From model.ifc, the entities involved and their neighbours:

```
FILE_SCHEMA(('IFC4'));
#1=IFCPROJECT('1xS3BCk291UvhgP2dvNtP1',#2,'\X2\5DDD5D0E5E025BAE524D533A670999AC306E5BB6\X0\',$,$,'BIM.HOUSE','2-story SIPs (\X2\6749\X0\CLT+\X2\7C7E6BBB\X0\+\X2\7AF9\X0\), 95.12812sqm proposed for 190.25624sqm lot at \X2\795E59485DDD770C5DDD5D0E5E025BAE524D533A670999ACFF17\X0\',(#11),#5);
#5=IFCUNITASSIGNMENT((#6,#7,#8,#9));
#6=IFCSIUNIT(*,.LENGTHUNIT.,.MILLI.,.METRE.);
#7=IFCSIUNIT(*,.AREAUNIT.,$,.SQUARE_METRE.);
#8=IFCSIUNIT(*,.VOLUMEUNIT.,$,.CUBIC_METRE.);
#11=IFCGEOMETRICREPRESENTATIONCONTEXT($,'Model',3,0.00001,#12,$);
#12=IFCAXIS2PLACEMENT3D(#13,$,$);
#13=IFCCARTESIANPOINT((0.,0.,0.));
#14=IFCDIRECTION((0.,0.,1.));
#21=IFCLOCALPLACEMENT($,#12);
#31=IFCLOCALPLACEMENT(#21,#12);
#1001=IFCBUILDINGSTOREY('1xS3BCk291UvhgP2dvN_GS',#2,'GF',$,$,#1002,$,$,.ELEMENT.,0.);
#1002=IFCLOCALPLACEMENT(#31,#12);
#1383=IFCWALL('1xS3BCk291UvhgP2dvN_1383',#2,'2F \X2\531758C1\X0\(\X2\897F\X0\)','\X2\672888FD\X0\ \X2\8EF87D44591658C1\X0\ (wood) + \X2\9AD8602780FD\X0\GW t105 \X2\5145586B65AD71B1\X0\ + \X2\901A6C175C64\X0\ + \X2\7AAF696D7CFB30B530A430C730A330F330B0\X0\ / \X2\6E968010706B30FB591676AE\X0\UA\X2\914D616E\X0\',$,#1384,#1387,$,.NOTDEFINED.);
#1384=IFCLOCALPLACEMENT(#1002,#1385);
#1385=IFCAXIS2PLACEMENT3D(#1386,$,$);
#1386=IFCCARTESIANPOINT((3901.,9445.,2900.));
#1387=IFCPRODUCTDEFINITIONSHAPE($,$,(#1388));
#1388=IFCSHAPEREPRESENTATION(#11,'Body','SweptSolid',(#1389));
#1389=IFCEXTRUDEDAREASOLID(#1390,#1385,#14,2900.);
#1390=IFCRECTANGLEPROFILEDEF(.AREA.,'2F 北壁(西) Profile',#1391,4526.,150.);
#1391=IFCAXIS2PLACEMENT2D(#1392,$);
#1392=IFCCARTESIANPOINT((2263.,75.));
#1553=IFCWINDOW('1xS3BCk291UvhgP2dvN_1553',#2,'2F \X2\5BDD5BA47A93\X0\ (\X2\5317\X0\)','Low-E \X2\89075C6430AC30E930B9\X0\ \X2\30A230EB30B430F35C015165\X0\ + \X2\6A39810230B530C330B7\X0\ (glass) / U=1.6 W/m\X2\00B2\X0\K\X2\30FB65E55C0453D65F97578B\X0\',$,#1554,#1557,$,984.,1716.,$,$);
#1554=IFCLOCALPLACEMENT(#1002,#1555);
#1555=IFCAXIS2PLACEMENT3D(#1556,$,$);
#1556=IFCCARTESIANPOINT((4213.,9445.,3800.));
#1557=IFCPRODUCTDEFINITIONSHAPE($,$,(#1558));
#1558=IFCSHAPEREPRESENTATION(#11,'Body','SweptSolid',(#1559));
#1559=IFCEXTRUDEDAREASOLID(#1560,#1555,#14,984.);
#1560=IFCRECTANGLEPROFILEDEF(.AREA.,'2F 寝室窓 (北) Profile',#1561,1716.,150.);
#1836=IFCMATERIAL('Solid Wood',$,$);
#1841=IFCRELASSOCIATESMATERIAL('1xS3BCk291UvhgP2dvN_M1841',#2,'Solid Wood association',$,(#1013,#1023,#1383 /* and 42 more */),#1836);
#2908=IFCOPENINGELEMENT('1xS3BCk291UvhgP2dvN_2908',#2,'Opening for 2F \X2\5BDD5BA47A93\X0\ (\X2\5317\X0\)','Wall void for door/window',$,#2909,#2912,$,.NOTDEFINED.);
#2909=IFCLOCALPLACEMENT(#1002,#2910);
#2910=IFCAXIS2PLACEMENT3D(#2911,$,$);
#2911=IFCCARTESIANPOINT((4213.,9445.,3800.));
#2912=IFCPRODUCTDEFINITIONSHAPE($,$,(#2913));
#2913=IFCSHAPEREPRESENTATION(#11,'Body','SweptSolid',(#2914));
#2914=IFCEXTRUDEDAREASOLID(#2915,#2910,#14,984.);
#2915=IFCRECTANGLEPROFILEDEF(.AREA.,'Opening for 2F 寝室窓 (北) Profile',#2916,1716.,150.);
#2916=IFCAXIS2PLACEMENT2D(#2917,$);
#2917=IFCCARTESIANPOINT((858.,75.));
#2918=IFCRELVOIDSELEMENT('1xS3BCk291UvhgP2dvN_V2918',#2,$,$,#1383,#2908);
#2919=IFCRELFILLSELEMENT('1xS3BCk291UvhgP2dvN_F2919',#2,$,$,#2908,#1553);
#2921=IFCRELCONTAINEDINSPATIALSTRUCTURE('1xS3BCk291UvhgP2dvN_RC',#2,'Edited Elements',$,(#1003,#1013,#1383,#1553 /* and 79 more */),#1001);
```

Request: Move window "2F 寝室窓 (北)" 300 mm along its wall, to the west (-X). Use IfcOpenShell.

```python
import ifcopenshell
import ifcopenshell.api.geometry
import ifcopenshell.util.placement
import ifcopenshell.util.unit

model = ifcopenshell.open("model.ifc")
unit_scale = ifcopenshell.util.unit.calculate_unit_scale(model)

window = model.by_guid("1xS3BCk291UvhgP2dvN_1553")
opening = window.FillsVoids[0].RelatingOpeningElement
wall = opening.VoidsElements[0].RelatingBuildingElement

wall_matrix = ifcopenshell.util.placement.get_local_placement(wall.ObjectPlacement)
shift = wall_matrix[:3, 0] * -0.3 / unit_scale
before = ifcopenshell.util.placement.get_local_placement(window.ObjectPlacement)[:3, 3].copy()

# The window is not placed relative to its opening, so move both.
for product in (opening, window):
    matrix = ifcopenshell.util.placement.get_local_placement(product.ObjectPlacement)
    matrix[:3, 3] += shift
    ifcopenshell.api.geometry.edit_object_placement(model, product=product, matrix=matrix, is_si=False)

after = ifcopenshell.util.placement.get_local_placement(window.ObjectPlacement)[:3, 3]
print("window moved by", (after - before).round(3) + 0.0)

model.write("model_v2.ifc")
```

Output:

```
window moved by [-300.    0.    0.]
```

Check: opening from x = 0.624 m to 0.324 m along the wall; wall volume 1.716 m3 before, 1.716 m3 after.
